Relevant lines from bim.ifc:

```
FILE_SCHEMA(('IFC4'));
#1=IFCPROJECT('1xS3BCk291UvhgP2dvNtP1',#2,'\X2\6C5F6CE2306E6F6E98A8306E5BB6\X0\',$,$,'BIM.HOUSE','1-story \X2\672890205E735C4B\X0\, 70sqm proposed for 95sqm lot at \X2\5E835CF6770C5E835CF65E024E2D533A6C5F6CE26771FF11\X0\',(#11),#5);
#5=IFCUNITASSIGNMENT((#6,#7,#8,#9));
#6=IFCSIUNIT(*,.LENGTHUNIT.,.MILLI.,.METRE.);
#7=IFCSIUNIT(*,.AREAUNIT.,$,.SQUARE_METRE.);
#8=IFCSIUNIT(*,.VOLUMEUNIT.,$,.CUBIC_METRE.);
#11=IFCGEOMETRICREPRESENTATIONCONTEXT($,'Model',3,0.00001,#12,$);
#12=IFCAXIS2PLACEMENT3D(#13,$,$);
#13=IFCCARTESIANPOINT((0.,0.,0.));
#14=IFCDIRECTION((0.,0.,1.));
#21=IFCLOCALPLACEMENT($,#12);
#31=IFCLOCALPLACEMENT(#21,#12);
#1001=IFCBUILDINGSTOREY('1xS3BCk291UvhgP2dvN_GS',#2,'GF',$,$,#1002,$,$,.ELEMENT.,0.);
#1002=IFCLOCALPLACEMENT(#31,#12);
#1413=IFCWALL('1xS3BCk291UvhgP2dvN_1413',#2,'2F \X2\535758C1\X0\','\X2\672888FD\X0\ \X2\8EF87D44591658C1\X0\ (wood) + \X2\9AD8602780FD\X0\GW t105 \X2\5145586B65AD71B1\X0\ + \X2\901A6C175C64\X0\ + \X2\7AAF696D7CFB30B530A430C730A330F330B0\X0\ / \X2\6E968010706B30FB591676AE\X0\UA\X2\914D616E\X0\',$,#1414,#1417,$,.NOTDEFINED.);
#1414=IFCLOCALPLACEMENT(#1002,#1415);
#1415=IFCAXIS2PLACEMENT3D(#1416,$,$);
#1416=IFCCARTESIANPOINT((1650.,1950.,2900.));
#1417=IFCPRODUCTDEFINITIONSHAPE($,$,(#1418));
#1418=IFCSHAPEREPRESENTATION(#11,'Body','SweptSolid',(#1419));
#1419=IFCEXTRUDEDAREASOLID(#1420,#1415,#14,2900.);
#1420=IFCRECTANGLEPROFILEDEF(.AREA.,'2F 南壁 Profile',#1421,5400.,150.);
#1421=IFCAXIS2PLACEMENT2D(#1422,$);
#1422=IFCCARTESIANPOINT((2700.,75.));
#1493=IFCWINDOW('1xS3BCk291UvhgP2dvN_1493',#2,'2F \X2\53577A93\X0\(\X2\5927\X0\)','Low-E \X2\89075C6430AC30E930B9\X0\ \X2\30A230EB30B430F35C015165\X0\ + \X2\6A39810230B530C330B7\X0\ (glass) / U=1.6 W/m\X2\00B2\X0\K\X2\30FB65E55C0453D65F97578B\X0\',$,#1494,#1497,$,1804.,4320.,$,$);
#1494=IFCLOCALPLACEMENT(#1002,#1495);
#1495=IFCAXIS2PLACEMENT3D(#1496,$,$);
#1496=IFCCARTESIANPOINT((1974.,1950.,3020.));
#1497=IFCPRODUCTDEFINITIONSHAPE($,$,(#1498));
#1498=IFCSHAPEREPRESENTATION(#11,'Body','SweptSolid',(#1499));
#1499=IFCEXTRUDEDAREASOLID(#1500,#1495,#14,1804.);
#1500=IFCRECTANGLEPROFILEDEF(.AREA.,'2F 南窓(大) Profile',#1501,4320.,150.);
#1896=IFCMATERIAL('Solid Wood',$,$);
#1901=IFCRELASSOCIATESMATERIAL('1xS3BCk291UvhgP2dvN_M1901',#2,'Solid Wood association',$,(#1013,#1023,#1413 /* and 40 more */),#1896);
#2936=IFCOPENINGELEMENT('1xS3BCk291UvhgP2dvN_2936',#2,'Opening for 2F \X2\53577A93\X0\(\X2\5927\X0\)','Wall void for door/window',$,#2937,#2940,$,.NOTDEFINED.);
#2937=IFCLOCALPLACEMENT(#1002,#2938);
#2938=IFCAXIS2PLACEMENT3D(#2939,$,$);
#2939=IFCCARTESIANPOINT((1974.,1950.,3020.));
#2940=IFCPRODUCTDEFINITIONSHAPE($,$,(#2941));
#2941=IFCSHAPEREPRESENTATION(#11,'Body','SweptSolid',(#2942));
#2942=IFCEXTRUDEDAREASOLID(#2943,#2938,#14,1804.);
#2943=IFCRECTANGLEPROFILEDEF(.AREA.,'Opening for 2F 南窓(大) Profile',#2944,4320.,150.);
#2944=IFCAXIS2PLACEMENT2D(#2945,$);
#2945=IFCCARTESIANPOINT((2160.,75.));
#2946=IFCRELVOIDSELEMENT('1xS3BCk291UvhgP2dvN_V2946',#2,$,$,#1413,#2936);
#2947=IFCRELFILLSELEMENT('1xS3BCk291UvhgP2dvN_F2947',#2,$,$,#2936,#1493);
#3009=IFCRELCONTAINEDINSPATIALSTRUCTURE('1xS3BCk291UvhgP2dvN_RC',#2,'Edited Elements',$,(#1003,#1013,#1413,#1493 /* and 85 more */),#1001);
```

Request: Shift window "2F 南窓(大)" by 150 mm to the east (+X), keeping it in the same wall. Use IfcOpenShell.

```python
import ifcopenshell
import ifcopenshell.api.geometry
import ifcopenshell.util.placement
import ifcopenshell.util.unit

model = ifcopenshell.open("bim.ifc")
unit_scale = ifcopenshell.util.unit.calculate_unit_scale(model)

window = model.by_guid("1xS3BCk291UvhgP2dvN_1493")
opening = window.FillsVoids[0].RelatingOpeningElement
wall = opening.VoidsElements[0].RelatingBuildingElement

wall_matrix = ifcopenshell.util.placement.get_local_placement(wall.ObjectPlacement)
shift = wall_matrix[:3, 0] * 0.15 / unit_scale
before = ifcopenshell.util.placement.get_local_placement(window.ObjectPlacement)[:3, 3].copy()

# The window is not placed relative to its opening, so move both.
for product in (opening, window):
    matrix = ifcopenshell.util.placement.get_local_placement(product.ObjectPlacement)
    matrix[:3, 3] += shift
    ifcopenshell.api.geometry.edit_object_placement(model, product=product, matrix=matrix, is_si=False)

after = ifcopenshell.util.placement.get_local_placement(window.ObjectPlacement)[:3, 3]
print("window moved by", (after - before).round(3) + 0.0)

model.write("bim_updated.ifc")
```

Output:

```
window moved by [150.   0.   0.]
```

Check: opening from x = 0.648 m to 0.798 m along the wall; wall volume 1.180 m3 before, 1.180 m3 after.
